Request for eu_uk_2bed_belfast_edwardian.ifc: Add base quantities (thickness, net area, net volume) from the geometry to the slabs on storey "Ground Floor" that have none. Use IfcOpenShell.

First a look at what the model holds.

```python
import ifcopenshell
import ifcopenshell.util.element
import ifcopenshell.util.unit

model = ifcopenshell.open("eu_uk_2bed_belfast_edwardian.ifc")
print(model.schema)
for unit_type in ("LENGTHUNIT", "AREAUNIT", "VOLUMEUNIT"):
    print(unit_type, ifcopenshell.util.unit.calculate_unit_scale(model, unit_type))
storey = next(s for s in model.by_type("IfcBuildingStorey") if s.Name == "Ground Floor")
slabs = [e for e in ifcopenshell.util.element.get_decomposition(storey) if e.is_a("IfcSlab")]
for e in sorted(slabs, key=lambda e: e.id()):
    print(e.id(), e.is_a(), e.Name, list(ifcopenshell.util.element.get_psets(e, qtos_only=True)), sep=" | ")
```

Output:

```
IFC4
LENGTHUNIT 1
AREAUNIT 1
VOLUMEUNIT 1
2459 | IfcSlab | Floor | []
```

```python
import ifcopenshell
import ifcopenshell.api.pset
import ifcopenshell.geom
import ifcopenshell.util.element
import ifcopenshell.util.shape
import ifcopenshell.util.unit

model = ifcopenshell.open("eu_uk_2bed_belfast_edwardian.ifc")
unit_scale = ifcopenshell.util.unit.calculate_unit_scale(model)
area_scale = ifcopenshell.util.unit.calculate_unit_scale(model, "AREAUNIT")
volume_scale = ifcopenshell.util.unit.calculate_unit_scale(model, "VOLUMEUNIT")
settings = ifcopenshell.geom.settings()

storey = next(s for s in model.by_type("IfcBuildingStorey") if s.Name == "Ground Floor")
slabs = [e for e in ifcopenshell.util.element.get_decomposition(storey) if e.is_a("IfcSlab")]

for e in sorted(slabs, key=lambda e: e.id()):
    if ifcopenshell.util.element.get_psets(e, qtos_only=True, should_inherit=False):
        continue
    # Geometry comes back in metres, in the element's own axes.
    shape = ifcopenshell.geom.create_shape(settings, e)
    values = {
        "Width": ifcopenshell.util.shape.get_z(shape.geometry) / unit_scale,
        "NetArea": ifcopenshell.util.shape.get_footprint_area(shape.geometry) / area_scale,
        "NetVolume": ifcopenshell.util.shape.get_volume(shape.geometry) / volume_scale,
    }
    qto = ifcopenshell.api.pset.add_qto(model, product=e, name="Qto_SlabBaseQuantities")
    ifcopenshell.api.pset.edit_qto(model, qto=qto, properties=values)
    print(e.id(), {k: round(v, 3) for k, v in values.items()})

model.write("eu_uk_2bed_belfast_edwardian_updated.ifc")
```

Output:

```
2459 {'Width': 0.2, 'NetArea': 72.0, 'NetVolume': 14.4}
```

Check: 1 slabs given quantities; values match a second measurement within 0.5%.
